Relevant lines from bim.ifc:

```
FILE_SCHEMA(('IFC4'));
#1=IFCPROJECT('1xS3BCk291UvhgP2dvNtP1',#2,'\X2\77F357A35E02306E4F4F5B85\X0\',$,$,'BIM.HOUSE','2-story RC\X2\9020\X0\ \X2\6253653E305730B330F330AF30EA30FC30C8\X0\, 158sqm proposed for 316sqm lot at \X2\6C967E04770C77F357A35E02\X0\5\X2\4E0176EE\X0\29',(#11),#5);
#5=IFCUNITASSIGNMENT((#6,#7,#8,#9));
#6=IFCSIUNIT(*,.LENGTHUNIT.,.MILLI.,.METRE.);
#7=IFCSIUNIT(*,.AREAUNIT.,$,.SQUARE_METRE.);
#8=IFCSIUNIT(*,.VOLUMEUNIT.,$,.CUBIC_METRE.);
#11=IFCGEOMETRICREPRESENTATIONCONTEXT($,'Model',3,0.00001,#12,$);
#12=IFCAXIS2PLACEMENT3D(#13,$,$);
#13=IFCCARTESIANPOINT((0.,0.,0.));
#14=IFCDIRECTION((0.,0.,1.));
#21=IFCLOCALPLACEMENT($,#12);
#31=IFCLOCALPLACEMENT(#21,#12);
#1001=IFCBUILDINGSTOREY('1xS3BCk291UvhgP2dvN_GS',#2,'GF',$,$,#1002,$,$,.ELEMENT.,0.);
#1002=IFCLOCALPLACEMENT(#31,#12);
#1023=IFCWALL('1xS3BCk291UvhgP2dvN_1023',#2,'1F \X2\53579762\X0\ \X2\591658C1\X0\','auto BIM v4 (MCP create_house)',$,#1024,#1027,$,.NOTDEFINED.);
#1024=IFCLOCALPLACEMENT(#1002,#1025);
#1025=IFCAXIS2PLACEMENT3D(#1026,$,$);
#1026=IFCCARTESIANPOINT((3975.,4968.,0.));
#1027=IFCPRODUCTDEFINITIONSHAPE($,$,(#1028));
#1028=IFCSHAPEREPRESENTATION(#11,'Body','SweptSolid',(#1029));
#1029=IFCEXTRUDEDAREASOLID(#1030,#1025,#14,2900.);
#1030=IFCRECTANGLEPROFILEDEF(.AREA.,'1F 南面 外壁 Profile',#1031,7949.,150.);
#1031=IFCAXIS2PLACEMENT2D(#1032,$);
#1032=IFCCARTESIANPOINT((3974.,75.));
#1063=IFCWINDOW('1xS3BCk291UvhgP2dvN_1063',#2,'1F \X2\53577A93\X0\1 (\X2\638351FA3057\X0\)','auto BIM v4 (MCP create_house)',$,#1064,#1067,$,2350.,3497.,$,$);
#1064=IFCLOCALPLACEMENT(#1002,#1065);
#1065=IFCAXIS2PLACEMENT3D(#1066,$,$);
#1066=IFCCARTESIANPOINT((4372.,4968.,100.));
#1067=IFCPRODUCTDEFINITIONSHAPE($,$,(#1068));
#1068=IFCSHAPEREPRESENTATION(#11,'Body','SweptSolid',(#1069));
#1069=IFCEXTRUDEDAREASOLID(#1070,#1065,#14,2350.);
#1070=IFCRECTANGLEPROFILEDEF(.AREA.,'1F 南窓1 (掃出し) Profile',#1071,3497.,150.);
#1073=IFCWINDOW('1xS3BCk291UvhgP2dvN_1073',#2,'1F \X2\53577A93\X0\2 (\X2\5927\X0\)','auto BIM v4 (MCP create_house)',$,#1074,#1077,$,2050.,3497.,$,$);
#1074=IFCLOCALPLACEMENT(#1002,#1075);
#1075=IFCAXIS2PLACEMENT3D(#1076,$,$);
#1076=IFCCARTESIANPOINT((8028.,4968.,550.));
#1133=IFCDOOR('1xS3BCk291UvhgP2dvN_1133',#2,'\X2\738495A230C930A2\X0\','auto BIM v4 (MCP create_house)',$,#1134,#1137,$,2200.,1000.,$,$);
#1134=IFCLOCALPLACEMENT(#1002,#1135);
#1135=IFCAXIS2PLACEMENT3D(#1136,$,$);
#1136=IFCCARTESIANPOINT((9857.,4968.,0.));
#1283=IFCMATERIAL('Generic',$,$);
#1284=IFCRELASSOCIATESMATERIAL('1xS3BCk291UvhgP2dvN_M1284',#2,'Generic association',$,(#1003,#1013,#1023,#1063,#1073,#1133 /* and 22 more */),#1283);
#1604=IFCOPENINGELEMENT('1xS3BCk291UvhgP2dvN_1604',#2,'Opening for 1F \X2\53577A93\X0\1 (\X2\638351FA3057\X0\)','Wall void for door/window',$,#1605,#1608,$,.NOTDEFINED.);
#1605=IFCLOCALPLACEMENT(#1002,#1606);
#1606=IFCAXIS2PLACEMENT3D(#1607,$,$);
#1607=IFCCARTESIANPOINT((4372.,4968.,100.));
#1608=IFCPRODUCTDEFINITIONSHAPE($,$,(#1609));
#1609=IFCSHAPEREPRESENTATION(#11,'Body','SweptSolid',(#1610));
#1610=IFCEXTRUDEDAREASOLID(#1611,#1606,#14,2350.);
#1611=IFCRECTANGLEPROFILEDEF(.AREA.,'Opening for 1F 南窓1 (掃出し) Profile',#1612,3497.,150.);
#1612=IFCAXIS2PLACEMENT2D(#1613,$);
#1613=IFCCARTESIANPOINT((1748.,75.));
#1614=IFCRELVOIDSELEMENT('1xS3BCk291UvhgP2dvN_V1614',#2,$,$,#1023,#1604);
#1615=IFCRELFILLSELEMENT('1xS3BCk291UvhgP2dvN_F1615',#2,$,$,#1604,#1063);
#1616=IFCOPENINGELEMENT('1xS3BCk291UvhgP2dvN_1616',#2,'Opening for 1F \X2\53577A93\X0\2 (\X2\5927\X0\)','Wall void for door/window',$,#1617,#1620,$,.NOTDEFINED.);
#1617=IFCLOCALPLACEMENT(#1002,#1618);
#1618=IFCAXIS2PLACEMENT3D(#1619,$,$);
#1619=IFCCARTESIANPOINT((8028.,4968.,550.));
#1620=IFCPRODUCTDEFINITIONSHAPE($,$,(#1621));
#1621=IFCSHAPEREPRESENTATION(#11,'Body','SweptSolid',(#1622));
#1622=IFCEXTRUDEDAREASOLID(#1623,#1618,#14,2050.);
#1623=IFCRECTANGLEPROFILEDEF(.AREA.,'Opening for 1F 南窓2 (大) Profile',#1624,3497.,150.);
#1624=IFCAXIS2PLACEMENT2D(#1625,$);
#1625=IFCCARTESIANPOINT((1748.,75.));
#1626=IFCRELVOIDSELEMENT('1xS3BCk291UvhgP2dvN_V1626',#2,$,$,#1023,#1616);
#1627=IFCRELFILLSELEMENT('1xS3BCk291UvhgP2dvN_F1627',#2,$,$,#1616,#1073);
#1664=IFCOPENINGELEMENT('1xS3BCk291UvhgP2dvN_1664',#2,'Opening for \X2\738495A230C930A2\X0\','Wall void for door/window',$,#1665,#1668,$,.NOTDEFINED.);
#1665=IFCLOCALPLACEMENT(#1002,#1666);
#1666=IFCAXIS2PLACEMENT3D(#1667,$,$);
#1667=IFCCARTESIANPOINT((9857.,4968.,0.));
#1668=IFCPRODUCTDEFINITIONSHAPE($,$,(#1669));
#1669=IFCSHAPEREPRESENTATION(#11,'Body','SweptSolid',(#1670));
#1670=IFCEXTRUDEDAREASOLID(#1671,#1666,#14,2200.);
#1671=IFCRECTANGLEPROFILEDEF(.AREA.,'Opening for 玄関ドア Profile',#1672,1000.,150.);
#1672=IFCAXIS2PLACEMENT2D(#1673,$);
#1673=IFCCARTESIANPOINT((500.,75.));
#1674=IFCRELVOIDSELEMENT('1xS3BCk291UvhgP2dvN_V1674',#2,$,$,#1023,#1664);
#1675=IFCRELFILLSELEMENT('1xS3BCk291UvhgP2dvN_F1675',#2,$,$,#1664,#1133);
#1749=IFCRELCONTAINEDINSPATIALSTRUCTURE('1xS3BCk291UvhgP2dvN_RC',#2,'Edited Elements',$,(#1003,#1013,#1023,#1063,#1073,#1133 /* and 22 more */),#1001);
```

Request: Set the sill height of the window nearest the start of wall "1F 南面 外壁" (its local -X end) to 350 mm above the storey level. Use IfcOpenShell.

```python
import numpy as np
import ifcopenshell
import ifcopenshell.api.geometry
import ifcopenshell.geom
import ifcopenshell.util.element
import ifcopenshell.util.placement
import ifcopenshell.util.shape
import ifcopenshell.util.unit

model = ifcopenshell.open("bim.ifc")
unit_scale = ifcopenshell.util.unit.calculate_unit_scale(model)

window = model.by_id(1063)
opening = window.FillsVoids[0].RelatingOpeningElement
storey = ifcopenshell.util.element.get_container(window, ifc_class="IfcBuildingStorey")
level = ifcopenshell.util.placement.get_local_placement(storey.ObjectPlacement)[2, 3]

# The opening's origin need not be at the sill, so measure its lowest point.
shape = ifcopenshell.geom.create_shape(ifcopenshell.geom.settings(), opening)
bottom = ifcopenshell.util.shape.get_shape_bottom_elevation(shape, shape.geometry) / unit_scale
dz = level + 0.35 / unit_scale - bottom

shift = np.array([0.0, 0.0, dz])
# The window is not placed relative to its opening, so move both.
for product in (opening, window):
    matrix = ifcopenshell.util.placement.get_local_placement(product.ObjectPlacement)
    matrix[:3, 3] += shift
    ifcopenshell.api.geometry.edit_object_placement(model, product=product, matrix=matrix, is_si=False)

print(f"moved by {dz * unit_scale:+.3f} m")

model.write("bim_edited.ifc")
```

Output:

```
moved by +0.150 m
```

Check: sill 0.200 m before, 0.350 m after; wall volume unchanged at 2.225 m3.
